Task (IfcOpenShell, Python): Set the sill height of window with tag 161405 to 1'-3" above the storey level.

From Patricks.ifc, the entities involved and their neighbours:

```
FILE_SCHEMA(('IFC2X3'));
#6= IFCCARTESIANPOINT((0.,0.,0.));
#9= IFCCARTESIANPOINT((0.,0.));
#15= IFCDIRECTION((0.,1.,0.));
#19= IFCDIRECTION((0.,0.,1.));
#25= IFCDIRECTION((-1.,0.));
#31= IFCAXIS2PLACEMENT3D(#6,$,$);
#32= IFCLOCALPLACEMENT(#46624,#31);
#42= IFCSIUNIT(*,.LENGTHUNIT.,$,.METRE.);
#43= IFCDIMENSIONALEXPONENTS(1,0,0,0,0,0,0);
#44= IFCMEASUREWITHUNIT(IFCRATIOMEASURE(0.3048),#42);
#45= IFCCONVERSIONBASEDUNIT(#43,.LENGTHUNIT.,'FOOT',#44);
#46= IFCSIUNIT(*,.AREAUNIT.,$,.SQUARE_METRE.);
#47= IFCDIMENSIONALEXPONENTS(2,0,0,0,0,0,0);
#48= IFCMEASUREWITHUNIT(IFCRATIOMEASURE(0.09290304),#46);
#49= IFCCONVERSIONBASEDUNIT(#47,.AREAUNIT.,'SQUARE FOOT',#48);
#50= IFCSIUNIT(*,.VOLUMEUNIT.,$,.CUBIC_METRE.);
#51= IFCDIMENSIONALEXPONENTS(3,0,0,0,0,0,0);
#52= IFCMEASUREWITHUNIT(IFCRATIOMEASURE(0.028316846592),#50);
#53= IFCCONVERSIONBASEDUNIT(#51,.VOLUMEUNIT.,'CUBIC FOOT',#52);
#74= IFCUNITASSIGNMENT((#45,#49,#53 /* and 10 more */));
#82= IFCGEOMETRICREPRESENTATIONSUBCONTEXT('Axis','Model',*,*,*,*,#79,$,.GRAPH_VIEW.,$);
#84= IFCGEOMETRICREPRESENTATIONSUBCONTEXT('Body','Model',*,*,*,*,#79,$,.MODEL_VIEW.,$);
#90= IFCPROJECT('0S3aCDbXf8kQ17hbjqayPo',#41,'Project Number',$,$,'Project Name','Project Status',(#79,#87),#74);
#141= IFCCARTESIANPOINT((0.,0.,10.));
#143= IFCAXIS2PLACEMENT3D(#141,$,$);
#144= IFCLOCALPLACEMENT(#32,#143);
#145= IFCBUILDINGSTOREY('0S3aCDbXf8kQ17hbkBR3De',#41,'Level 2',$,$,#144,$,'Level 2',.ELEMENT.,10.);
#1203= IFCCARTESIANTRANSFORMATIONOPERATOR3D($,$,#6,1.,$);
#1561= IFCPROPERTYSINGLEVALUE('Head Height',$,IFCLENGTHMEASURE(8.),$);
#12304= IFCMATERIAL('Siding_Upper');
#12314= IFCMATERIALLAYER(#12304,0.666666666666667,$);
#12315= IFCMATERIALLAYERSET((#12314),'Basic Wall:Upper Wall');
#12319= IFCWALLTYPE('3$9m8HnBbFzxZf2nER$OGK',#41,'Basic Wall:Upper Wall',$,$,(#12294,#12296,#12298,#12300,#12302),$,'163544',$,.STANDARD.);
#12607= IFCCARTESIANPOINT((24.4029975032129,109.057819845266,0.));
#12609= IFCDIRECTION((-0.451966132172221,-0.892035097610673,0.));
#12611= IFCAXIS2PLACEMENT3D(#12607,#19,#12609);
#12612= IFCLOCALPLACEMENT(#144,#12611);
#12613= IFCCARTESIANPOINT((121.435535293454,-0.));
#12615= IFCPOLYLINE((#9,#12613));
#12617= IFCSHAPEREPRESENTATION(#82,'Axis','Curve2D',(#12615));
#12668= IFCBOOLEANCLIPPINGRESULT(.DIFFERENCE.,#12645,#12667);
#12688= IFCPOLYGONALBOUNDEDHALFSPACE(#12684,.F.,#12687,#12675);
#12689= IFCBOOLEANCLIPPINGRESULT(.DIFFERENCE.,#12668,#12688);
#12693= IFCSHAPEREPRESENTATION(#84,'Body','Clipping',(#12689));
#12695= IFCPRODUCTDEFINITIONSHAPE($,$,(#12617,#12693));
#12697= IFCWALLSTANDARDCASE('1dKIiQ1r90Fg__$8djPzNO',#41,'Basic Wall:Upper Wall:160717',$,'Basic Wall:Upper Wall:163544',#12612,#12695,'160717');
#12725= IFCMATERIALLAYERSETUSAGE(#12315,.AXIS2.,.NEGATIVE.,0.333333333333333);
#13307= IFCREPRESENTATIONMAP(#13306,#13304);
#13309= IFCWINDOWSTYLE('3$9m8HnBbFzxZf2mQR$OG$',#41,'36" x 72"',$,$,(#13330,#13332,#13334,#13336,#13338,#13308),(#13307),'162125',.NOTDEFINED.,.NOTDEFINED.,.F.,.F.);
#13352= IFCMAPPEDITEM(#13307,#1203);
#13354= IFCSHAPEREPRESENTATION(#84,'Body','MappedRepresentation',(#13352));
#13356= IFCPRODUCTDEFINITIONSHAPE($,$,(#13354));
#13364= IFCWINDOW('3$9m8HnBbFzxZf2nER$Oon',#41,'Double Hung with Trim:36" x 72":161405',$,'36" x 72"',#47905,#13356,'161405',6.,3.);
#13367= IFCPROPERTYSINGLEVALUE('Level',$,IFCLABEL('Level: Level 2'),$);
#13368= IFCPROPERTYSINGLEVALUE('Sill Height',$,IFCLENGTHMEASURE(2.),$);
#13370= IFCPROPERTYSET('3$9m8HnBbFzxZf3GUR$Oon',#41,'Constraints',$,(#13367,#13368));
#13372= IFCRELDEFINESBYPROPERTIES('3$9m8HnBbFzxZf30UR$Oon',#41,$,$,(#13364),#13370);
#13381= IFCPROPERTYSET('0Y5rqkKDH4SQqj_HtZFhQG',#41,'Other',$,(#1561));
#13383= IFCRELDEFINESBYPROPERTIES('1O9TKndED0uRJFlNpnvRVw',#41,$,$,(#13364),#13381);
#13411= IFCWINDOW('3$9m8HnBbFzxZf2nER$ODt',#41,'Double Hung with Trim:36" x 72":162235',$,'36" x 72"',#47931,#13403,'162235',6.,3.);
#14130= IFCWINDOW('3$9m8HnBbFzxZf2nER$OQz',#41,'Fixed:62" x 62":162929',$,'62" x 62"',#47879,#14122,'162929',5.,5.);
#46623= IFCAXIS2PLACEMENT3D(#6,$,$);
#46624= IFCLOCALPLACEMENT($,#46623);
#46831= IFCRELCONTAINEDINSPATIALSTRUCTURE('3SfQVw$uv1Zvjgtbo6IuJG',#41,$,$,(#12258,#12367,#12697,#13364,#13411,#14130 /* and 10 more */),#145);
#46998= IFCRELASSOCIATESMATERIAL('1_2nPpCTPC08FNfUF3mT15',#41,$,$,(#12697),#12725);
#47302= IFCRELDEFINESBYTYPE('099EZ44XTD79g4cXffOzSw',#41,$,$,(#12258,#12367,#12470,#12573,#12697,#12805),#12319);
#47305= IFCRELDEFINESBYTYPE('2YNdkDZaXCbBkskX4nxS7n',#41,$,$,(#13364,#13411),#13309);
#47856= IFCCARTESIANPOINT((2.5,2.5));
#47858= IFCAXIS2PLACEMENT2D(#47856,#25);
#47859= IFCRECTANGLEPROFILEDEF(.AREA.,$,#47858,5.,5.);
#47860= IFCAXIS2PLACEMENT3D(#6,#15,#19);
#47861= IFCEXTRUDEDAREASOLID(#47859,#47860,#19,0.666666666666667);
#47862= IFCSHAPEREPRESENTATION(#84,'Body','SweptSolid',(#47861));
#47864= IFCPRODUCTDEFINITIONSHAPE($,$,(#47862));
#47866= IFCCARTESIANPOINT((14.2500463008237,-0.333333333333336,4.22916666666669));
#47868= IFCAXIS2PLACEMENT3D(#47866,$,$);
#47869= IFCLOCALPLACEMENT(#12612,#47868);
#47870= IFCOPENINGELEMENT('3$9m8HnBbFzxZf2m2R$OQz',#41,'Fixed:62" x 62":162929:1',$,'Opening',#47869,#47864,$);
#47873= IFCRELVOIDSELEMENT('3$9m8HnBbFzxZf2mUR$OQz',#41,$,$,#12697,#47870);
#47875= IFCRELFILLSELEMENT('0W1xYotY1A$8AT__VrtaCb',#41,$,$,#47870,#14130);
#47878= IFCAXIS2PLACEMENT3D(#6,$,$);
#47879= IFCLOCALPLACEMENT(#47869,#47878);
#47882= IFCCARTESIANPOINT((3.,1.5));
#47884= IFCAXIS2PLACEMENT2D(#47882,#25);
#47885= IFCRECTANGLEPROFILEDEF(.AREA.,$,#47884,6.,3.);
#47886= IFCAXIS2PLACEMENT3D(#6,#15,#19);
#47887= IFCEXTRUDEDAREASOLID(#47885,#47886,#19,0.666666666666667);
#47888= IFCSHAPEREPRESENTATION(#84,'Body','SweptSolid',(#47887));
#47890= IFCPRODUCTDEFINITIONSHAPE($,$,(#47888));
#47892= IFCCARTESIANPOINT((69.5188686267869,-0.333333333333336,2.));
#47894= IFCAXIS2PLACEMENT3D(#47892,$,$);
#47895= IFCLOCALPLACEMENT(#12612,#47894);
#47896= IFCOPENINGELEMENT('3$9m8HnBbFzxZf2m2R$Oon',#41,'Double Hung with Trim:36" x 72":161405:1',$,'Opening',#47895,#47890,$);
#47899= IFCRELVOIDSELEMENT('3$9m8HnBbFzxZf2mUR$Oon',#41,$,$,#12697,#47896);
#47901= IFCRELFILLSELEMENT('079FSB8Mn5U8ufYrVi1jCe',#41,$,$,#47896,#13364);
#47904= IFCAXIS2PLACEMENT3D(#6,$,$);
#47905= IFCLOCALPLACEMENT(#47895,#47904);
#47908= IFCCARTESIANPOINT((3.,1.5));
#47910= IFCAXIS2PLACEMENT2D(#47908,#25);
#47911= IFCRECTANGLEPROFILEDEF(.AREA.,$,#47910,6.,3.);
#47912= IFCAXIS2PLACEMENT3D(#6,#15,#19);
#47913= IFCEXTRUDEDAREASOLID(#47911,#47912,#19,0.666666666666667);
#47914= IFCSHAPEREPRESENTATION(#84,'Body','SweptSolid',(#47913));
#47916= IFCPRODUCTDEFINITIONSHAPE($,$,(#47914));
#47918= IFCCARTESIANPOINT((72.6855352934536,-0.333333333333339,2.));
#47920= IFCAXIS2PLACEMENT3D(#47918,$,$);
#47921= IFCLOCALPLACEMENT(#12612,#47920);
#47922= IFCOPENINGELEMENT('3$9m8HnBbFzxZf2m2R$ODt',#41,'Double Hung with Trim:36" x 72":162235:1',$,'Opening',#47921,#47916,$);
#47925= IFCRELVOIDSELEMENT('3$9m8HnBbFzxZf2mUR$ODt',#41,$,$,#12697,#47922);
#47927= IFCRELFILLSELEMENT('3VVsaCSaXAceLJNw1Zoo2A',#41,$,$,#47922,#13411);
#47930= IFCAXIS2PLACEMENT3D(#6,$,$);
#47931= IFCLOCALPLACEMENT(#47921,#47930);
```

```python
import numpy as np
import ifcopenshell
import ifcopenshell.api.geometry
import ifcopenshell.api.pset
import ifcopenshell.geom
import ifcopenshell.util.element
import ifcopenshell.util.placement
import ifcopenshell.util.shape
import ifcopenshell.util.unit

model = ifcopenshell.open("Patricks.ifc")
unit_scale = ifcopenshell.util.unit.calculate_unit_scale(model)

window = model.by_guid("3$9m8HnBbFzxZf2nER$Oon")
opening = window.FillsVoids[0].RelatingOpeningElement
storey = ifcopenshell.util.element.get_container(window, ifc_class="IfcBuildingStorey")
level = ifcopenshell.util.placement.get_local_placement(storey.ObjectPlacement)[2, 3]

# The opening's origin need not be at the sill, so measure its lowest point.
shape = ifcopenshell.geom.create_shape(ifcopenshell.geom.settings(), opening)
bottom = ifcopenshell.util.shape.get_shape_bottom_elevation(shape, shape.geometry) / unit_scale
dz = level + 15 * 0.0254 / unit_scale - bottom

shift = np.array([0.0, 0.0, dz])
# The window is placed relative to its opening, so it follows when the opening moves.
matrix = ifcopenshell.util.placement.get_local_placement(opening.ObjectPlacement)
matrix[:3, 3] += shift
ifcopenshell.api.geometry.edit_object_placement(
    model, product=opening, matrix=matrix, is_si=False, should_transform_children=True
)

# Keep the stored heights in step.
pset = model.by_id(ifcopenshell.util.element.get_pset(window, "Constraints", should_inherit=False)["id"])
ifcopenshell.api.pset.edit_pset(model, pset=pset, properties={
    "Sill Height": model.create_entity("IfcLengthMeasure", ifcopenshell.util.element.get_pset(window, "Constraints", "Sill Height") + dz),
})
pset = model.by_id(ifcopenshell.util.element.get_pset(window, "Other", should_inherit=False)["id"])
ifcopenshell.api.pset.edit_pset(model, pset=pset, properties={
    "Head Height": model.create_entity("IfcLengthMeasure", ifcopenshell.util.element.get_pset(window, "Other", "Head Height") + dz),
})

print(f"moved by {dz * unit_scale:+.3f} m")

model.write("Patricks-out.ifc")
```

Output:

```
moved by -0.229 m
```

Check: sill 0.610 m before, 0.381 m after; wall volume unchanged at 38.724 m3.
